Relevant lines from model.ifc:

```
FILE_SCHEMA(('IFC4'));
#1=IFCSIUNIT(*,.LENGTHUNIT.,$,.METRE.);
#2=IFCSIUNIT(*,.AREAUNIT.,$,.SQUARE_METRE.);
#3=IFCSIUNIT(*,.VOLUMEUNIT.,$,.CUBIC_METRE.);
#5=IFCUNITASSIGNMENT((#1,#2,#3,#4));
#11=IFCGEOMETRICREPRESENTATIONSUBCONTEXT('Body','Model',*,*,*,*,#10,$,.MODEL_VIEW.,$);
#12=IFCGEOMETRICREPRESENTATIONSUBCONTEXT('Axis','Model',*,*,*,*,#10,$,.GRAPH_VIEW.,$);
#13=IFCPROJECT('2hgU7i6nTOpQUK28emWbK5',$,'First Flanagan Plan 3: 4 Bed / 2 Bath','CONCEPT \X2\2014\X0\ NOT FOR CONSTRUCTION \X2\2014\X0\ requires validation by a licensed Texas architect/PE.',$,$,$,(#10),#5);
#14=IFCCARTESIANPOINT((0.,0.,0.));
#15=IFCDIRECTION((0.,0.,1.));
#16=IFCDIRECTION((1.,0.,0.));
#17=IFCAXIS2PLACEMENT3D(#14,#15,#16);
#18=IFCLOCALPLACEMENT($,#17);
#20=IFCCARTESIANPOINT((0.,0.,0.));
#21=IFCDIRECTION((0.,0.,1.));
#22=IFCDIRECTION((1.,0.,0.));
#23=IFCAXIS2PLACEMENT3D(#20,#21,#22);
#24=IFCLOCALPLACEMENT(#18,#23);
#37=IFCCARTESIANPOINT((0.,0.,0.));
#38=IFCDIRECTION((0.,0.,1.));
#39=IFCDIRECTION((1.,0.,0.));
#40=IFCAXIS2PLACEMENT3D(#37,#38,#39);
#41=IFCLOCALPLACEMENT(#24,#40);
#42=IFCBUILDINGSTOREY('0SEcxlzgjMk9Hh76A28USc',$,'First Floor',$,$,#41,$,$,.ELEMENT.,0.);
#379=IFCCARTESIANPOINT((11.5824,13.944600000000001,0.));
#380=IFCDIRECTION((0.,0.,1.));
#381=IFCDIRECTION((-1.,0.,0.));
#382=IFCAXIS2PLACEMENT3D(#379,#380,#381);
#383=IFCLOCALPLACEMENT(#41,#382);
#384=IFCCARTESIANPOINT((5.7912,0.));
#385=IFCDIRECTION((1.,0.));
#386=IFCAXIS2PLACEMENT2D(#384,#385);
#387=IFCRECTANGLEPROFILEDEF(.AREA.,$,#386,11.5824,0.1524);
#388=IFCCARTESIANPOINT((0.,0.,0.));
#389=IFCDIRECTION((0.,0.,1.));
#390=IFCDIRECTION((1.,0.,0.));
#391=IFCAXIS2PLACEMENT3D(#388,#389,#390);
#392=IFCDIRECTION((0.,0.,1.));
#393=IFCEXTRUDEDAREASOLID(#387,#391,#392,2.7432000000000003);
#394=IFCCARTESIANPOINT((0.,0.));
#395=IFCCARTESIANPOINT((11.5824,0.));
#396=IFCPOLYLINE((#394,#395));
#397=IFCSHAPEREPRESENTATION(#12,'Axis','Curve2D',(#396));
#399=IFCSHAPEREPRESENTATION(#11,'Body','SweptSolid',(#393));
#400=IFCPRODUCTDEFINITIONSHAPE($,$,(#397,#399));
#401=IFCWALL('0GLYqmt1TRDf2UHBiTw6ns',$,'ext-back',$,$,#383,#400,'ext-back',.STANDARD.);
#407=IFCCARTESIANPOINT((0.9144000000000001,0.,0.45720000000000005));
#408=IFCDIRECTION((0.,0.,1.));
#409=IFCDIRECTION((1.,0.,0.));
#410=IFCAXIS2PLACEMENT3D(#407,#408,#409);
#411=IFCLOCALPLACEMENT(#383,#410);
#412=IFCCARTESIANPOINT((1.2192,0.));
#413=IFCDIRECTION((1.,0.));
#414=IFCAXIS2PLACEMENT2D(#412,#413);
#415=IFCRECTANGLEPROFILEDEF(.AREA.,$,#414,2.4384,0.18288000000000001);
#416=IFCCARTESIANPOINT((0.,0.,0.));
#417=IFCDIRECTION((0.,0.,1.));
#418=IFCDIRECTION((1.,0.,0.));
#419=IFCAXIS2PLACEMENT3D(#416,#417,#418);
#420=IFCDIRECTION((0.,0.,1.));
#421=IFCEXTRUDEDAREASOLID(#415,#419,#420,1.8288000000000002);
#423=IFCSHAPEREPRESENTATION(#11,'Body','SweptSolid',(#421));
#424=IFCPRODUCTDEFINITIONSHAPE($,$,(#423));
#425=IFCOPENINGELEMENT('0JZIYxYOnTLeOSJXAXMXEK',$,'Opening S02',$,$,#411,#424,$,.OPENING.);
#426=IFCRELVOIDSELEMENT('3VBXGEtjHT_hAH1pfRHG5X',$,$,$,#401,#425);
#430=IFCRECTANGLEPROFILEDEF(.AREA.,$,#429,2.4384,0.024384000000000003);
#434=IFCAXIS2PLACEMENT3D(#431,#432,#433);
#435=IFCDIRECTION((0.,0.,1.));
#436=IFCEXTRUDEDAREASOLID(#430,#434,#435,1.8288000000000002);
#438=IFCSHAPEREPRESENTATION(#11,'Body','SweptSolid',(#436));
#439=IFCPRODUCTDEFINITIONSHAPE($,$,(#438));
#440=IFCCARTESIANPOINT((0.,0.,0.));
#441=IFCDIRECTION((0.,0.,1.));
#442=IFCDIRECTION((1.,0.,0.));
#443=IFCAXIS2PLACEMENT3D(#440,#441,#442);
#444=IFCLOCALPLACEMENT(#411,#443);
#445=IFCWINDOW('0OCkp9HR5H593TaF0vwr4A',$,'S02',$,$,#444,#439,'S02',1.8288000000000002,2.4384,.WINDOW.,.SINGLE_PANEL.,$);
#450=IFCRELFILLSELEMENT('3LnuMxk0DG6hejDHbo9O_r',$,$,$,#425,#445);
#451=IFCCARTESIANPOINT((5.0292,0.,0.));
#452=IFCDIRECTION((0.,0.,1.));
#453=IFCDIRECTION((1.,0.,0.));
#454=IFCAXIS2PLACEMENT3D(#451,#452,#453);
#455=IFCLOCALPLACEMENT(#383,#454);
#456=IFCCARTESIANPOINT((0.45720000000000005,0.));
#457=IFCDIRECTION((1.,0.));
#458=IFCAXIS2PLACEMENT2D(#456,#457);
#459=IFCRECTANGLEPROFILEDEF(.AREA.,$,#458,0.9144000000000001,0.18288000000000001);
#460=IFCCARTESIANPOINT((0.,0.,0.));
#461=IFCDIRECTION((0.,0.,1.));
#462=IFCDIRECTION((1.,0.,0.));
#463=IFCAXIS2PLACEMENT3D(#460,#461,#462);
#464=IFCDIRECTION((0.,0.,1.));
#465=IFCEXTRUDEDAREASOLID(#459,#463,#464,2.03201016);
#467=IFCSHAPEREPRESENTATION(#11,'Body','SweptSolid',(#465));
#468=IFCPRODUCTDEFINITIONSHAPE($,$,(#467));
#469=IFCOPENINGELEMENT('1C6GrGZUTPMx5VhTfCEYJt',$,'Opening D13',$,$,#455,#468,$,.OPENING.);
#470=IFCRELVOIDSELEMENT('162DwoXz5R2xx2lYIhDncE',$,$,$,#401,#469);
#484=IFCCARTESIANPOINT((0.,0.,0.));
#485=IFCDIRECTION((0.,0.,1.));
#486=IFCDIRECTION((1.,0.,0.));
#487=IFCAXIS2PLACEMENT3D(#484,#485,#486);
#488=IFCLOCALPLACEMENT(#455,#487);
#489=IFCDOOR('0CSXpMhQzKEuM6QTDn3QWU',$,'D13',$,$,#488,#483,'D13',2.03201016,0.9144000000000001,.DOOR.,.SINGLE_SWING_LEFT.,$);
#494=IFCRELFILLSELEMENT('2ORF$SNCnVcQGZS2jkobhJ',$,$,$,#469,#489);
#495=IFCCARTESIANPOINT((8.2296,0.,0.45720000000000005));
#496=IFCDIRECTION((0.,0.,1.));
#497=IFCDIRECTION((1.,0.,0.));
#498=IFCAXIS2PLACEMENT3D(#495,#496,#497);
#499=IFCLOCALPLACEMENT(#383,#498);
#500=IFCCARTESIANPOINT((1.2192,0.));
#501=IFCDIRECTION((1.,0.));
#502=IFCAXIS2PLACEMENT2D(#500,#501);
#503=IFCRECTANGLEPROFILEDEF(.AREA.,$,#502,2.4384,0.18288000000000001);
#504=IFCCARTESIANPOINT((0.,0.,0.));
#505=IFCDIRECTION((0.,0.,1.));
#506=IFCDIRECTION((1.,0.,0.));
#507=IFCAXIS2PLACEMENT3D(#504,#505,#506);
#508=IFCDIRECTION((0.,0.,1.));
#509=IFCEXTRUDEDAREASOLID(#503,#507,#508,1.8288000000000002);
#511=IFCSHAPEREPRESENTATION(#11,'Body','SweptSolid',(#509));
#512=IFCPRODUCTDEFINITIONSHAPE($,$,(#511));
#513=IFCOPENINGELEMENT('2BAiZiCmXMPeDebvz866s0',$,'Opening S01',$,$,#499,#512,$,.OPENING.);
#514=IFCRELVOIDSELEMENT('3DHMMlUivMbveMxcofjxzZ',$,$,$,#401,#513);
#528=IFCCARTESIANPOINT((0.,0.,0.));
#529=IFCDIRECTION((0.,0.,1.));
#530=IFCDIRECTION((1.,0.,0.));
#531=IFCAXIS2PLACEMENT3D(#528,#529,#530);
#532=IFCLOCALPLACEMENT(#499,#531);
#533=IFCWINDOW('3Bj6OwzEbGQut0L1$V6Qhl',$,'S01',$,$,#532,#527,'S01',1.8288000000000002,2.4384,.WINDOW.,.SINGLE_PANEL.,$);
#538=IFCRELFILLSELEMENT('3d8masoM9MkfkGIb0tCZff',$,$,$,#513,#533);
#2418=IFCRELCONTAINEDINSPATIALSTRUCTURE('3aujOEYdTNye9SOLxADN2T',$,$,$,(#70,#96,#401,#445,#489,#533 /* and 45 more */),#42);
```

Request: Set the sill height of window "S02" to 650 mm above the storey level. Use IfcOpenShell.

```python
import numpy as np
import ifcopenshell
import ifcopenshell.api.geometry
import ifcopenshell.geom
import ifcopenshell.util.element
import ifcopenshell.util.placement
import ifcopenshell.util.shape
import ifcopenshell.util.unit

model = ifcopenshell.open("model.ifc")
unit_scale = ifcopenshell.util.unit.calculate_unit_scale(model)

window = model.by_guid("0OCkp9HR5H593TaF0vwr4A")
opening = window.FillsVoids[0].RelatingOpeningElement
storey = ifcopenshell.util.element.get_container(window, ifc_class="IfcBuildingStorey")
level = ifcopenshell.util.placement.get_local_placement(storey.ObjectPlacement)[2, 3]

# The opening's origin need not be at the sill, so measure its lowest point.
shape = ifcopenshell.geom.create_shape(ifcopenshell.geom.settings(), opening)
bottom = ifcopenshell.util.shape.get_shape_bottom_elevation(shape, shape.geometry) / unit_scale
dz = level + 0.65 / unit_scale - bottom

shift = np.array([0.0, 0.0, dz])
# The window is placed relative to its opening, so it follows when the opening moves.
matrix = ifcopenshell.util.placement.get_local_placement(opening.ObjectPlacement)
matrix[:3, 3] += shift
ifcopenshell.api.geometry.edit_object_placement(
    model, product=opening, matrix=matrix, is_si=False, should_transform_children=True
)

print(f"moved by {dz * unit_scale:+.3f} m")

model.write("model_edited.ifc")
```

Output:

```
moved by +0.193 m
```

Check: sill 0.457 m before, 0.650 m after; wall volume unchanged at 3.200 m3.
